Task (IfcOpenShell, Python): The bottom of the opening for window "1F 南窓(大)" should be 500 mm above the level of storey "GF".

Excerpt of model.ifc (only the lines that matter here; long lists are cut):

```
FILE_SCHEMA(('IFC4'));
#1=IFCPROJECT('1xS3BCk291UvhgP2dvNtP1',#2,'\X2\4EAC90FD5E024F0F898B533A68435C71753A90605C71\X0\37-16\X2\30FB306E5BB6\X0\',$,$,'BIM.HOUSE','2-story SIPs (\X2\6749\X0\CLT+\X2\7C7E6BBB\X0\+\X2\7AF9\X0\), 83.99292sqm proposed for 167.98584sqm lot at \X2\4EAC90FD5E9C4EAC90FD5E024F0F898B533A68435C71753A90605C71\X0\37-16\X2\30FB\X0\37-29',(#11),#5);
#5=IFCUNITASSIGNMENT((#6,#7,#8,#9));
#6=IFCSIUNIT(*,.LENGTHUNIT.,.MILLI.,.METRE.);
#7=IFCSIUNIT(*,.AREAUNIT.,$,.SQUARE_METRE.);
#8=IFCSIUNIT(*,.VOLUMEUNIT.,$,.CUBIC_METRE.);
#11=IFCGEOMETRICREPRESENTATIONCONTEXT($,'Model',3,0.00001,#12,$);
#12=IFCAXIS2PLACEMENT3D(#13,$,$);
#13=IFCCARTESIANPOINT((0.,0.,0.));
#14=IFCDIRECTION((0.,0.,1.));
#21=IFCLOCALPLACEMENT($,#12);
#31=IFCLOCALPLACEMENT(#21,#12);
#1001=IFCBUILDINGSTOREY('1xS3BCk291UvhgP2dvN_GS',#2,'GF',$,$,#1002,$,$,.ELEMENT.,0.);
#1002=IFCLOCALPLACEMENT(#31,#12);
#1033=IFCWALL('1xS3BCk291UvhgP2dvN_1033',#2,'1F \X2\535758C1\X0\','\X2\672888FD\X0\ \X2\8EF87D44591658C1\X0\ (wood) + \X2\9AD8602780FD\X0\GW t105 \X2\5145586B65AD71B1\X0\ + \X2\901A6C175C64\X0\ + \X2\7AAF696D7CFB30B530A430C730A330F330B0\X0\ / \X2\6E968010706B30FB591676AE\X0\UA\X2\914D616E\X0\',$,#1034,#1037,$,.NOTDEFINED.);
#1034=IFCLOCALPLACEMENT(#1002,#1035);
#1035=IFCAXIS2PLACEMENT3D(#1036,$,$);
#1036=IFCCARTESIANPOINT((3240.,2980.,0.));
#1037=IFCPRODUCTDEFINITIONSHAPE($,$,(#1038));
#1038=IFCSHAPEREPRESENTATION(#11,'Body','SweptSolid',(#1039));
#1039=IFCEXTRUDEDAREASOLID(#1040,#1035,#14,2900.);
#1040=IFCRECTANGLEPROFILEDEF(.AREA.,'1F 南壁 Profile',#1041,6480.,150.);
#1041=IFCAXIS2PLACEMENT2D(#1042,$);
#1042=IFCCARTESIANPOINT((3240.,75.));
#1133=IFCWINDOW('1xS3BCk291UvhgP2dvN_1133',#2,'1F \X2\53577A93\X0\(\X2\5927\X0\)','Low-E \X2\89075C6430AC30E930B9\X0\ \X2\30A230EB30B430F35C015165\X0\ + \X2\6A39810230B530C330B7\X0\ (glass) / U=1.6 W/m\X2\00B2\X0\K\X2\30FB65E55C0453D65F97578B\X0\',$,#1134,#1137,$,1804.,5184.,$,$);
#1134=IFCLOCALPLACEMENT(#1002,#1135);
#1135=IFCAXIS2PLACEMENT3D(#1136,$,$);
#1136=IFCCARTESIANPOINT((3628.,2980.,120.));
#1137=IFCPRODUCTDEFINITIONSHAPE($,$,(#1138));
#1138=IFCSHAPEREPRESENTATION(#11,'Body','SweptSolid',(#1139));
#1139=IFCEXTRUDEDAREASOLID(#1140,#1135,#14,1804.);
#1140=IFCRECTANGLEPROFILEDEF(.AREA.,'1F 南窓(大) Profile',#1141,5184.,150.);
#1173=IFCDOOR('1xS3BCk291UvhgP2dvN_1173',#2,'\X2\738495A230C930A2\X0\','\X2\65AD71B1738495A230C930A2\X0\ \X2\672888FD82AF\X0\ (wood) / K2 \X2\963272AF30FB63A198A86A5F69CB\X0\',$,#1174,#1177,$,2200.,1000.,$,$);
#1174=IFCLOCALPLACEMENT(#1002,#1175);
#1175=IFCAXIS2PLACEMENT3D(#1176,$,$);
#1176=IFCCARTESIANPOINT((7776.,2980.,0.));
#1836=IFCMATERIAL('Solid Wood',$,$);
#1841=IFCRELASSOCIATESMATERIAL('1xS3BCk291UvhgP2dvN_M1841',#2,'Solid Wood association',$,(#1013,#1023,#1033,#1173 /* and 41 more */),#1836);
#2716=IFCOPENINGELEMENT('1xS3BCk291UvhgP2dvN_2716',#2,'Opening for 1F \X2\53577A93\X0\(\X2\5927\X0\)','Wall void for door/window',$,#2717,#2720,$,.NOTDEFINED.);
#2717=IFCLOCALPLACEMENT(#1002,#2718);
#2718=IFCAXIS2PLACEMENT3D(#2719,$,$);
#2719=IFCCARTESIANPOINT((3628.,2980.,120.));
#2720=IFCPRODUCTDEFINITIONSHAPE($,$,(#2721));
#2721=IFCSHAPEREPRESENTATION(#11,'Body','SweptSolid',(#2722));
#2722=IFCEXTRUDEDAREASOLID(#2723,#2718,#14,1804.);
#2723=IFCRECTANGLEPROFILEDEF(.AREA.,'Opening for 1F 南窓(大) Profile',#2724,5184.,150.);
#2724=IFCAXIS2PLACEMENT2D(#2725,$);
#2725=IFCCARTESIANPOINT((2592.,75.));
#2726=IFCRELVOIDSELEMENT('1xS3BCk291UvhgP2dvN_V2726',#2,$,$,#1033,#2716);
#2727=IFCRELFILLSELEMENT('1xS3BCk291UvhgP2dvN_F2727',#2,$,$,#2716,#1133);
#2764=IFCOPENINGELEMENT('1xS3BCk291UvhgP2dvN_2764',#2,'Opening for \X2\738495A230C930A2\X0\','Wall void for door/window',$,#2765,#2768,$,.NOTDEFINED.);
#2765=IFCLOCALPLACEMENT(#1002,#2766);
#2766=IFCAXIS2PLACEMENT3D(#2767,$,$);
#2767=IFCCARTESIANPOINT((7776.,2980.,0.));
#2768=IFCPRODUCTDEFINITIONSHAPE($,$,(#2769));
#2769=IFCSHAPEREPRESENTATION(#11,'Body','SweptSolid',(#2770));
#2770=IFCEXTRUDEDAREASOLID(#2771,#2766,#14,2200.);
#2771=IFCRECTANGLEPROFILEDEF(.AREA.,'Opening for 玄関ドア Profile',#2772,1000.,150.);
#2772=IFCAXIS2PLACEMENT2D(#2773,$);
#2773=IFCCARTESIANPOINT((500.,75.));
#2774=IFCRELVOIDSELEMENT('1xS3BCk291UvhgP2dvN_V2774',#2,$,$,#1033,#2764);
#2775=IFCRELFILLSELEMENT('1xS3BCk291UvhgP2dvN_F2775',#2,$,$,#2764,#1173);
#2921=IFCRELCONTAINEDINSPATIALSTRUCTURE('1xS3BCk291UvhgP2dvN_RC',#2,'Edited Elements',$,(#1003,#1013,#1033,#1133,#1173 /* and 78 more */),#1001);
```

```python
import numpy as np
import ifcopenshell
import ifcopenshell.api.geometry
import ifcopenshell.geom
import ifcopenshell.util.element
import ifcopenshell.util.placement
import ifcopenshell.util.shape
import ifcopenshell.util.unit

model = ifcopenshell.open("model.ifc")
unit_scale = ifcopenshell.util.unit.calculate_unit_scale(model)

window = model.by_guid("1xS3BCk291UvhgP2dvN_1133")
opening = window.FillsVoids[0].RelatingOpeningElement
storey = ifcopenshell.util.element.get_container(window, ifc_class="IfcBuildingStorey")
level = ifcopenshell.util.placement.get_local_placement(storey.ObjectPlacement)[2, 3]

# The opening's origin need not be at the sill, so measure its lowest point.
shape = ifcopenshell.geom.create_shape(ifcopenshell.geom.settings(), opening)
bottom = ifcopenshell.util.shape.get_shape_bottom_elevation(shape, shape.geometry) / unit_scale
dz = level + 0.5 / unit_scale - bottom

shift = np.array([0.0, 0.0, dz])
# The window is not placed relative to its opening, so move both.
for product in (opening, window):
    matrix = ifcopenshell.util.placement.get_local_placement(product.ObjectPlacement)
    matrix[:3, 3] += shift
    ifcopenshell.api.geometry.edit_object_placement(model, product=product, matrix=matrix, is_si=False)

print(f"moved by {dz * unit_scale:+.3f} m")

model.write("model_edited.ifc")
```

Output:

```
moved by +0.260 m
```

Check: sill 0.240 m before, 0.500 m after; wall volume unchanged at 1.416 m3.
